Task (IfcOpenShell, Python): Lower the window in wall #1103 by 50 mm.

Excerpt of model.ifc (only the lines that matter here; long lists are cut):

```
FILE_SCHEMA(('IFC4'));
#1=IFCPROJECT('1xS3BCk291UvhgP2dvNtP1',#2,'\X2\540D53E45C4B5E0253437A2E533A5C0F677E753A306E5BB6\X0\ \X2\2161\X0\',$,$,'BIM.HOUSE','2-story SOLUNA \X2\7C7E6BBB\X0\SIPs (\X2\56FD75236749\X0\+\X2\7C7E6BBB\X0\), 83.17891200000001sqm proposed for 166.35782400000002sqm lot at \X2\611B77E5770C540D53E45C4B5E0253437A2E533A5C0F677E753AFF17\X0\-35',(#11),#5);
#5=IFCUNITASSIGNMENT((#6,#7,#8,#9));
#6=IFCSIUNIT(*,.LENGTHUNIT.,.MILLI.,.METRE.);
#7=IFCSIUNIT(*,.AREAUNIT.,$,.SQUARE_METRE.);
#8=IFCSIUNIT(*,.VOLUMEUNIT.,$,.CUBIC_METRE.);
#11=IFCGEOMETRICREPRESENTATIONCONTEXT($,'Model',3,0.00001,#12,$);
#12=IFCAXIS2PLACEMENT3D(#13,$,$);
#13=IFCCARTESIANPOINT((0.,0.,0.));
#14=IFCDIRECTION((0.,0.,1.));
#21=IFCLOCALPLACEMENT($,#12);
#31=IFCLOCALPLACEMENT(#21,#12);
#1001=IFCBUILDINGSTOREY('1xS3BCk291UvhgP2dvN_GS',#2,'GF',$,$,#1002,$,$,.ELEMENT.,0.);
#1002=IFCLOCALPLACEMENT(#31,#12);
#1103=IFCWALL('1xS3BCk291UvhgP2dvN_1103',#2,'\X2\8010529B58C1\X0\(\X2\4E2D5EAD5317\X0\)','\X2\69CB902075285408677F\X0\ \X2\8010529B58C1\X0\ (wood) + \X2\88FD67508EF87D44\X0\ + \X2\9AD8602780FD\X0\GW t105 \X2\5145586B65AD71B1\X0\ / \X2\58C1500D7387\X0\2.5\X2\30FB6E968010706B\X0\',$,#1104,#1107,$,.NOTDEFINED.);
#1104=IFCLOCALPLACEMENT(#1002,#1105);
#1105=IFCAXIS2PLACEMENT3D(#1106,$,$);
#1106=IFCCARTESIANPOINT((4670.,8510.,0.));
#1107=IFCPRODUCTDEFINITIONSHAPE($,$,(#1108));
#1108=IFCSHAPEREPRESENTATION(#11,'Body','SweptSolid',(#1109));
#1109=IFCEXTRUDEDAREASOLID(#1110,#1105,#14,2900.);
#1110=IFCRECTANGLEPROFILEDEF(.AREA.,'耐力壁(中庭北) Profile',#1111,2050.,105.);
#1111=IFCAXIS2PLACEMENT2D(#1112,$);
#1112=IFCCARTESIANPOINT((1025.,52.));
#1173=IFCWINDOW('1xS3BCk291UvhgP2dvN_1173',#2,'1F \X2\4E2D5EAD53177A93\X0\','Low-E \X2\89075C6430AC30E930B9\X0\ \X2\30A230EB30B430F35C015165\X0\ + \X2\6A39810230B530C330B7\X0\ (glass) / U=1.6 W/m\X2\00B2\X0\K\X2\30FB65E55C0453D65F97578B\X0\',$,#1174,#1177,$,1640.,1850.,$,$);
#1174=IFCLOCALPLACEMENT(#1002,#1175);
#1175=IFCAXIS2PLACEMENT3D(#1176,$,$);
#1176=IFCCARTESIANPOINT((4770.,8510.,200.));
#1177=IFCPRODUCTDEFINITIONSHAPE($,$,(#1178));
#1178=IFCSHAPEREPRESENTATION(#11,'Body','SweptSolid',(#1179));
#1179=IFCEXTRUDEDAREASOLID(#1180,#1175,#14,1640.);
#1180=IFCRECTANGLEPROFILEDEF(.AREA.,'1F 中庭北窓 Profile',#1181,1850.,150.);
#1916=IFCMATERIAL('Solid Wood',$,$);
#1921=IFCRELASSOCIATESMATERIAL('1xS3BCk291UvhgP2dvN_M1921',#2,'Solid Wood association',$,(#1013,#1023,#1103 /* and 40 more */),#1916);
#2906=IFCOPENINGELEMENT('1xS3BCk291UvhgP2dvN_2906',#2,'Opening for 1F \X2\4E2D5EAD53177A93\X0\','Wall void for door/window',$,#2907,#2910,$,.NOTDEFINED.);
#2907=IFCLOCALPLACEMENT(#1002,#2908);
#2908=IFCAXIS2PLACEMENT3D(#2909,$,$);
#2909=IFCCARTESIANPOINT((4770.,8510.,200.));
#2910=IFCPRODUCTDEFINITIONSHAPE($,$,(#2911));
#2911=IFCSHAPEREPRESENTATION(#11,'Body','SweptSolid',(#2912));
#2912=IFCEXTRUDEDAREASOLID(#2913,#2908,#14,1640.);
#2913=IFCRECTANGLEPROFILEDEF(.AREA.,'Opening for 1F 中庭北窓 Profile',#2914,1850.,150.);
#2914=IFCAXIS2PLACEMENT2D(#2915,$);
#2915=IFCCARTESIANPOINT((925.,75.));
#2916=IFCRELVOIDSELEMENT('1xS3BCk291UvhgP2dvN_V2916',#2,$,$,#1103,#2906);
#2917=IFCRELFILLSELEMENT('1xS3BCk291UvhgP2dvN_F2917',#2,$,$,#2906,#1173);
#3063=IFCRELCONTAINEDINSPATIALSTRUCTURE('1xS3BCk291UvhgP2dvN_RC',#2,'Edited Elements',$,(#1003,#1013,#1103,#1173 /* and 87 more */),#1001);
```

```python
import numpy as np
import ifcopenshell
import ifcopenshell.api.geometry
import ifcopenshell.util.placement
import ifcopenshell.util.unit

model = ifcopenshell.open("model.ifc")
unit_scale = ifcopenshell.util.unit.calculate_unit_scale(model)

window = model.by_id(1173)
opening = window.FillsVoids[0].RelatingOpeningElement
dz = -0.05 / unit_scale

shift = np.array([0.0, 0.0, dz])
# The window is not placed relative to its opening, so move both.
for product in (opening, window):
    matrix = ifcopenshell.util.placement.get_local_placement(product.ObjectPlacement)
    matrix[:3, 3] += shift
    ifcopenshell.api.geometry.edit_object_placement(model, product=product, matrix=matrix, is_si=False)

print(f"moved by {dz * unit_scale:+.3f} m")

model.write("model_edited.ifc")
```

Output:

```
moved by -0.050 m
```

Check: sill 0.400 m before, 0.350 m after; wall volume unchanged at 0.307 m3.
